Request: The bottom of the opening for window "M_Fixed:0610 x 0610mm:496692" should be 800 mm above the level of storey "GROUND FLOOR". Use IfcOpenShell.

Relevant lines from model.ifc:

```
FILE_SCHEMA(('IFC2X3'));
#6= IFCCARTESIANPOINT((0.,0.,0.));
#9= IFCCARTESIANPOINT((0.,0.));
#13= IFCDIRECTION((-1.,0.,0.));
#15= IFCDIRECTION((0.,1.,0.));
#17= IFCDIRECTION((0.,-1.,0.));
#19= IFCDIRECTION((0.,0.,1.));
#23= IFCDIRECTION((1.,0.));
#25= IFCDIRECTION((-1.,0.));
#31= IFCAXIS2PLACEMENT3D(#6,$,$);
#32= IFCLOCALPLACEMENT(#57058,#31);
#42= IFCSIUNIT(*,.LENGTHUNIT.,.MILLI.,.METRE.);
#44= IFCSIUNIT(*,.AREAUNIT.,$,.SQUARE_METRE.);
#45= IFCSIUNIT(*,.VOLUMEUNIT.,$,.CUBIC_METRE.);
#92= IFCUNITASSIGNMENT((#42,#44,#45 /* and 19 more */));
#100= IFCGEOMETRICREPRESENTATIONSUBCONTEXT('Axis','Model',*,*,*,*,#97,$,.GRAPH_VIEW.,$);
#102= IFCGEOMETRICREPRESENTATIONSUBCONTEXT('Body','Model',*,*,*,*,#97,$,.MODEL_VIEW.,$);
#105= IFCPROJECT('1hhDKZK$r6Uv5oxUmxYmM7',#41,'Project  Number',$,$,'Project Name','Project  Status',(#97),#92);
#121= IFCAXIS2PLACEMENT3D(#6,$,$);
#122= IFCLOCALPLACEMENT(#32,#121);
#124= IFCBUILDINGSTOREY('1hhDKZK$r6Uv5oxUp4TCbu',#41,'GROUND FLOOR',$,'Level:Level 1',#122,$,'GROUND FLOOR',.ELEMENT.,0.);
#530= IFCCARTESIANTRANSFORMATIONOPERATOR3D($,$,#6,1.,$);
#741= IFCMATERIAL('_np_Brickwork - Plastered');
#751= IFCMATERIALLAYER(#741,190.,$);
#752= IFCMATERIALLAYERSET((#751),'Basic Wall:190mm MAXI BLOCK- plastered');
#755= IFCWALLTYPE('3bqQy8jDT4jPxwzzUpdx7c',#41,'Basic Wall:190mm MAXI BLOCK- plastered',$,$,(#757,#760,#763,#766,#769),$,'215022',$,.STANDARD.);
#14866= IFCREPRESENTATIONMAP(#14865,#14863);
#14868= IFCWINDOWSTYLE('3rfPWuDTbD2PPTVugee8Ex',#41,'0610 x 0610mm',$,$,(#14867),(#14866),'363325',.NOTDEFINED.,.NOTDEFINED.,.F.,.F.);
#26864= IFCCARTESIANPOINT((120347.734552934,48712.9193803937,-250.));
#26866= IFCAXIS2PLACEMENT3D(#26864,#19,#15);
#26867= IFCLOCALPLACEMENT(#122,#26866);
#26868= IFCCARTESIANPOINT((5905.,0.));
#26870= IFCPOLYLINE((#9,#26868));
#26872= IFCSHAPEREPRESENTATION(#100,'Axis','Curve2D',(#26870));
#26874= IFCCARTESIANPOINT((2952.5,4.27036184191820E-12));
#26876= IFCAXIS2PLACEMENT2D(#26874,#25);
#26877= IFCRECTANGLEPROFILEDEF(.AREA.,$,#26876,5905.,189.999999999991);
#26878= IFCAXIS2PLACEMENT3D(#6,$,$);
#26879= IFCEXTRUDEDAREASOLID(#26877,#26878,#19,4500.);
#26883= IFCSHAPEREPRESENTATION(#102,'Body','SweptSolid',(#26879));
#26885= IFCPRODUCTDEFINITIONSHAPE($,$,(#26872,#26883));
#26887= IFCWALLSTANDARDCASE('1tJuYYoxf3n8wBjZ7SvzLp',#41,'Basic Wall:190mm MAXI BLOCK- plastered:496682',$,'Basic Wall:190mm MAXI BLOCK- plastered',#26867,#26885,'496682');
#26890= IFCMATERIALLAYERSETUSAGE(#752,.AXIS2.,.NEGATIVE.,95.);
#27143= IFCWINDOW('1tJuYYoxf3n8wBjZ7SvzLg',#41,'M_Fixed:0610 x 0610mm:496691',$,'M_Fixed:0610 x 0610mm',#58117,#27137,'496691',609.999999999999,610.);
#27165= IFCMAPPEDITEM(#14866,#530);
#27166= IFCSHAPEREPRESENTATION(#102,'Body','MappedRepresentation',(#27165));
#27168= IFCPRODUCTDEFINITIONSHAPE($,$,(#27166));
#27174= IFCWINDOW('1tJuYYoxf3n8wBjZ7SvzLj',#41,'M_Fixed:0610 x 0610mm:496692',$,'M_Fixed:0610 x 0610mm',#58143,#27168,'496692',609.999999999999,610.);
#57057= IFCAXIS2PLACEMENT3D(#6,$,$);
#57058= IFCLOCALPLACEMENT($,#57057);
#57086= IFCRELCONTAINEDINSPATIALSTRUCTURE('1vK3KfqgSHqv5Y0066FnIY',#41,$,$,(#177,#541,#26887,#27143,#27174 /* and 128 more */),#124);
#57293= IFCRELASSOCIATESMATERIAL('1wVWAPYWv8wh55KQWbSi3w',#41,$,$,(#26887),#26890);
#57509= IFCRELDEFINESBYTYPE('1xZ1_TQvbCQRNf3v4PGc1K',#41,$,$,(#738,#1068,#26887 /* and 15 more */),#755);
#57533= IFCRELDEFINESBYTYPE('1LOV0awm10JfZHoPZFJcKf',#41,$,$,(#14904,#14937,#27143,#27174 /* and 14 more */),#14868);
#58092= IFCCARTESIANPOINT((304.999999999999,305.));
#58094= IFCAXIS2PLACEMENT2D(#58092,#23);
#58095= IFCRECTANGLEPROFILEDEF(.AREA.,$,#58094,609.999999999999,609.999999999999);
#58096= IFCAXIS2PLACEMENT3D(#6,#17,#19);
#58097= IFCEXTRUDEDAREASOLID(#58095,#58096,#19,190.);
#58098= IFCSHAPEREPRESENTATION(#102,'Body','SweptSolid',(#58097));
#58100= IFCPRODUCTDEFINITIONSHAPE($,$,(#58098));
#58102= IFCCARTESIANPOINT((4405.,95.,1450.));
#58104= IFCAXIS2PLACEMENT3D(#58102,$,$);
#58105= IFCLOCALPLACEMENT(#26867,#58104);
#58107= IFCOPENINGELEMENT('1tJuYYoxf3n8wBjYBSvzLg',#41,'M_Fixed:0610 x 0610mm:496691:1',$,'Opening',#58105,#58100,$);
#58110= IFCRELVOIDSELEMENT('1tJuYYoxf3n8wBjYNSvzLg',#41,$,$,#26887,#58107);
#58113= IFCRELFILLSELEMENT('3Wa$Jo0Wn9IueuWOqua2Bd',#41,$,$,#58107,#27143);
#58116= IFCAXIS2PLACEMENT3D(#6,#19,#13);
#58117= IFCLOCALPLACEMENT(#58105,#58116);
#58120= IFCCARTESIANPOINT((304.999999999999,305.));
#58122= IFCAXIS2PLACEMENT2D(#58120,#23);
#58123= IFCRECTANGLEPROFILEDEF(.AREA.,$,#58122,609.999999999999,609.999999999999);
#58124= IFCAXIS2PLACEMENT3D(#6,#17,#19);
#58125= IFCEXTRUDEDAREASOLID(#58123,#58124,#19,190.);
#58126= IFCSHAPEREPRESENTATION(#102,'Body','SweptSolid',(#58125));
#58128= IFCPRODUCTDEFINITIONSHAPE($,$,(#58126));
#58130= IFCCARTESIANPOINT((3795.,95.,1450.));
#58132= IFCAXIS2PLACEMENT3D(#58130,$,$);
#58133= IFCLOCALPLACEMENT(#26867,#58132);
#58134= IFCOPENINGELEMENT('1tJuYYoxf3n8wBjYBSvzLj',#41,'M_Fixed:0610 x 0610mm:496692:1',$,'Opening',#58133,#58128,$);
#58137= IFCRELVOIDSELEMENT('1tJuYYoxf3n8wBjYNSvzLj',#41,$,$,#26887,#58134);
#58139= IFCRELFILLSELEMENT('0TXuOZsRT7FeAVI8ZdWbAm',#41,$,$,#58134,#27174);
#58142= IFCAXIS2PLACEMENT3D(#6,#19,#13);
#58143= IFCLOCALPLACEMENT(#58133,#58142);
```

```python
import numpy as np
import ifcopenshell
import ifcopenshell.api.geometry
import ifcopenshell.geom
import ifcopenshell.util.element
import ifcopenshell.util.placement
import ifcopenshell.util.shape
import ifcopenshell.util.unit

model = ifcopenshell.open("model.ifc")
unit_scale = ifcopenshell.util.unit.calculate_unit_scale(model)

window = model.by_id(27174)
opening = window.FillsVoids[0].RelatingOpeningElement
storey = ifcopenshell.util.element.get_container(window, ifc_class="IfcBuildingStorey")
level = ifcopenshell.util.placement.get_local_placement(storey.ObjectPlacement)[2, 3]

# The opening's origin need not be at the sill, so measure its lowest point.
shape = ifcopenshell.geom.create_shape(ifcopenshell.geom.settings(), opening)
bottom = ifcopenshell.util.shape.get_shape_bottom_elevation(shape, shape.geometry) / unit_scale
dz = level + 800.0 - bottom

shift = np.array([0.0, 0.0, dz])
# The window is placed relative to its opening, so it follows when the opening moves.
matrix = ifcopenshell.util.placement.get_local_placement(opening.ObjectPlacement)
matrix[:3, 3] += shift
ifcopenshell.api.geometry.edit_object_placement(
    model, product=opening, matrix=matrix, is_si=False, should_transform_children=True
)

print(f"moved by {dz * unit_scale:+.3f} m")

model.write("model-out.ifc")
```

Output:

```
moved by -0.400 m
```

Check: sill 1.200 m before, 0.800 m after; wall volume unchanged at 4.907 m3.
